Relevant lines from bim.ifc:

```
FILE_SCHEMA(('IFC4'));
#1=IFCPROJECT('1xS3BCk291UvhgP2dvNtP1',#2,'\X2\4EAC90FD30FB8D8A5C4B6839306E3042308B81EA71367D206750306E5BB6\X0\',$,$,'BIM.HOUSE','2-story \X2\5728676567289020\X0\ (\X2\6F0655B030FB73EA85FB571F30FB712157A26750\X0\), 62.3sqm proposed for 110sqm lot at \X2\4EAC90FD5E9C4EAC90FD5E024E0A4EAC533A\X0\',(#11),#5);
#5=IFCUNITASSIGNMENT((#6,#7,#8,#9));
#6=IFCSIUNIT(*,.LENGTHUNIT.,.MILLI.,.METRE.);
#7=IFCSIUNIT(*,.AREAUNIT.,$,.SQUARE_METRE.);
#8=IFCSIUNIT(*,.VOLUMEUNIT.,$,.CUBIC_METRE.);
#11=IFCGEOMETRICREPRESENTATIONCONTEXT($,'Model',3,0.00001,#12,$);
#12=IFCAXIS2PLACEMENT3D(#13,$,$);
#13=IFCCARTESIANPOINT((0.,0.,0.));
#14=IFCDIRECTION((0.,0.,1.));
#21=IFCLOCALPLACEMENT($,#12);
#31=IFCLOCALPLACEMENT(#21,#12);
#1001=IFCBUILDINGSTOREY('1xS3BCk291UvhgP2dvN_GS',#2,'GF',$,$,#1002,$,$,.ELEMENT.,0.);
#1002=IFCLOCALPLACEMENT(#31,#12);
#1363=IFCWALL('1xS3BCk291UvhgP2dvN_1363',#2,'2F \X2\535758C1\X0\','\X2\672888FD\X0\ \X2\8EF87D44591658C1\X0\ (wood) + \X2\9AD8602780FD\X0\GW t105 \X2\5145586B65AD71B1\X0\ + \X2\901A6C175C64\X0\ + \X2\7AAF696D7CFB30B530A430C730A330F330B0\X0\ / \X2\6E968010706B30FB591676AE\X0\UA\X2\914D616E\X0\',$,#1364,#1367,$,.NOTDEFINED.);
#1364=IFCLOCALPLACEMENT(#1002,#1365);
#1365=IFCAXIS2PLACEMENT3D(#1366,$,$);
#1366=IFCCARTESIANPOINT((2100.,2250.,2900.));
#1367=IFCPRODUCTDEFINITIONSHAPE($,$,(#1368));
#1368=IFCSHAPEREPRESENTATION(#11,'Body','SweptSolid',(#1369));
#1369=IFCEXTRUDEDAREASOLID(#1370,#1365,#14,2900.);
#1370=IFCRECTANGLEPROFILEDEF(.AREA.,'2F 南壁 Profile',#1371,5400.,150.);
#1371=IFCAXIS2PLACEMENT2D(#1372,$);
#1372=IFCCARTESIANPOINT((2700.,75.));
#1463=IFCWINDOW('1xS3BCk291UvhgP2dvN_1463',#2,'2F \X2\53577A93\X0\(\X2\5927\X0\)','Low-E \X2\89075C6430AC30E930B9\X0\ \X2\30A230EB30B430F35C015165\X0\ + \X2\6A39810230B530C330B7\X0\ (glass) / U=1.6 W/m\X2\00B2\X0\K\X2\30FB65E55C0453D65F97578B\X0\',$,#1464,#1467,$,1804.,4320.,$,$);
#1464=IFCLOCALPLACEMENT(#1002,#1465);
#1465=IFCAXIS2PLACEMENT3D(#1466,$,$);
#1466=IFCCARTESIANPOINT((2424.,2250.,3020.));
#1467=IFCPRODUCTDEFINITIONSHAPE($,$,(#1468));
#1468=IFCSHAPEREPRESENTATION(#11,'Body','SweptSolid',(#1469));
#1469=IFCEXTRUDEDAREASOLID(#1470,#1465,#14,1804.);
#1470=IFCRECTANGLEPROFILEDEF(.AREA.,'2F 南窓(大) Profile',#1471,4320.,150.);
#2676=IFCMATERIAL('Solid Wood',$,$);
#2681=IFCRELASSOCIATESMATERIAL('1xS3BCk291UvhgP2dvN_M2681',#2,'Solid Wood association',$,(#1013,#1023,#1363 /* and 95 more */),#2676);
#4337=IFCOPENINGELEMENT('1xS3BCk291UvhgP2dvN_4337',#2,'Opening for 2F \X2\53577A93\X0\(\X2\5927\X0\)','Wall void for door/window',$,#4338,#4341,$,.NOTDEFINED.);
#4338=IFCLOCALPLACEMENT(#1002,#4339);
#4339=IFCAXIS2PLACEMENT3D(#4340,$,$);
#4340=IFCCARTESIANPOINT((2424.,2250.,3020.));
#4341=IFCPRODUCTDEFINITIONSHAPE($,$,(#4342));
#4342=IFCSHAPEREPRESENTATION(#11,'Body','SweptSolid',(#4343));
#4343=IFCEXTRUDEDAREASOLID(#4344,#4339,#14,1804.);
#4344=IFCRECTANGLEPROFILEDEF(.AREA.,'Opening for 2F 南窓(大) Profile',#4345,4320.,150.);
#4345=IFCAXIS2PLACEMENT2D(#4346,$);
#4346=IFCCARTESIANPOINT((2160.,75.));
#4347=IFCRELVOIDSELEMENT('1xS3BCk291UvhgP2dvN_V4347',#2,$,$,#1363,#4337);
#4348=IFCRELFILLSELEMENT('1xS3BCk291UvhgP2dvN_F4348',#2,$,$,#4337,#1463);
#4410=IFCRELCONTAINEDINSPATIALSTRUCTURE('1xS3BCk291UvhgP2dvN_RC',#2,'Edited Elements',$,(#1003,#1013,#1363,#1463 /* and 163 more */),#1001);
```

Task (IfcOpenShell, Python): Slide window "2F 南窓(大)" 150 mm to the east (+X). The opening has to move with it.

```python
import ifcopenshell
import ifcopenshell.api.geometry
import ifcopenshell.util.placement

model = ifcopenshell.open("bim.ifc")

window = model.by_guid("1xS3BCk291UvhgP2dvN_1463")
opening = window.FillsVoids[0].RelatingOpeningElement
wall = opening.VoidsElements[0].RelatingBuildingElement

wall_matrix = ifcopenshell.util.placement.get_local_placement(wall.ObjectPlacement)
shift = wall_matrix[:3, 0] * 150.0
before = ifcopenshell.util.placement.get_local_placement(window.ObjectPlacement)[:3, 3].copy()

# The window is not placed relative to its opening, so move both.
for product in (opening, window):
    matrix = ifcopenshell.util.placement.get_local_placement(product.ObjectPlacement)
    matrix[:3, 3] += shift
    ifcopenshell.api.geometry.edit_object_placement(model, product=product, matrix=matrix, is_si=False)

after = ifcopenshell.util.placement.get_local_placement(window.ObjectPlacement)[:3, 3]
print("window moved by", (after - before).round(3) + 0.0)

model.write("bim_rev.ifc")
```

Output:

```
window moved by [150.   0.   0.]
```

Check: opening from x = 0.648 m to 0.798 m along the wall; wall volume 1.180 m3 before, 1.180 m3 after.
